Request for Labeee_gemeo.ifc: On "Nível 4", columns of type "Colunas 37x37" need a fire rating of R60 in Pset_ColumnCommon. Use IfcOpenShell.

First a look at what the model holds.

```python
import ifcopenshell
import ifcopenshell.util.element

model = ifcopenshell.open("Labeee_gemeo.ifc")
print(model.schema)
storey = next(s for s in model.by_type("IfcBuildingStorey") if s.Name == "Nível 4")
columns = [e for e in ifcopenshell.util.element.get_decomposition(storey) if e.is_a("IfcColumn")]
seen = {}
for e in columns:
    element_type = ifcopenshell.util.element.get_type(e)
    key = (element_type.Name if element_type != e and element_type else None, ifcopenshell.util.element.get_pset(e, "Pset_ColumnCommon", "FireRating"))
    seen[key] = seen.get(key, 0) + 1
for (name, value), count in sorted(seen.items(), key=str):
    print(count, "x", name, "|", value)
```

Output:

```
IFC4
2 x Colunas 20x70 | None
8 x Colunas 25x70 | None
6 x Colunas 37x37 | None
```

```python
import ifcopenshell
import ifcopenshell.api.pset
import ifcopenshell.util.element

model = ifcopenshell.open("Labeee_gemeo.ifc")

storey = next(s for s in model.by_type("IfcBuildingStorey") if s.Name == "Nível 4")
columns = [e for e in ifcopenshell.util.element.get_decomposition(storey) if e.is_a("IfcColumn")]

count = 0
for e in columns:
    element_type = ifcopenshell.util.element.get_type(e)
    if element_type in (None, e) or element_type.Name != "Colunas 37x37":
        continue
    # add_pset returns the element's existing set when there is one.
    pset = ifcopenshell.api.pset.add_pset(model, product=e, name="Pset_ColumnCommon")
    ifcopenshell.api.pset.edit_pset(model, pset=pset, properties={"FireRating": "R60"})
    count += 1

print(count, "columns updated")

model.write("Labeee_gemeo_updated.ifc")
```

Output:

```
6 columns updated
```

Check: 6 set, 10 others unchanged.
